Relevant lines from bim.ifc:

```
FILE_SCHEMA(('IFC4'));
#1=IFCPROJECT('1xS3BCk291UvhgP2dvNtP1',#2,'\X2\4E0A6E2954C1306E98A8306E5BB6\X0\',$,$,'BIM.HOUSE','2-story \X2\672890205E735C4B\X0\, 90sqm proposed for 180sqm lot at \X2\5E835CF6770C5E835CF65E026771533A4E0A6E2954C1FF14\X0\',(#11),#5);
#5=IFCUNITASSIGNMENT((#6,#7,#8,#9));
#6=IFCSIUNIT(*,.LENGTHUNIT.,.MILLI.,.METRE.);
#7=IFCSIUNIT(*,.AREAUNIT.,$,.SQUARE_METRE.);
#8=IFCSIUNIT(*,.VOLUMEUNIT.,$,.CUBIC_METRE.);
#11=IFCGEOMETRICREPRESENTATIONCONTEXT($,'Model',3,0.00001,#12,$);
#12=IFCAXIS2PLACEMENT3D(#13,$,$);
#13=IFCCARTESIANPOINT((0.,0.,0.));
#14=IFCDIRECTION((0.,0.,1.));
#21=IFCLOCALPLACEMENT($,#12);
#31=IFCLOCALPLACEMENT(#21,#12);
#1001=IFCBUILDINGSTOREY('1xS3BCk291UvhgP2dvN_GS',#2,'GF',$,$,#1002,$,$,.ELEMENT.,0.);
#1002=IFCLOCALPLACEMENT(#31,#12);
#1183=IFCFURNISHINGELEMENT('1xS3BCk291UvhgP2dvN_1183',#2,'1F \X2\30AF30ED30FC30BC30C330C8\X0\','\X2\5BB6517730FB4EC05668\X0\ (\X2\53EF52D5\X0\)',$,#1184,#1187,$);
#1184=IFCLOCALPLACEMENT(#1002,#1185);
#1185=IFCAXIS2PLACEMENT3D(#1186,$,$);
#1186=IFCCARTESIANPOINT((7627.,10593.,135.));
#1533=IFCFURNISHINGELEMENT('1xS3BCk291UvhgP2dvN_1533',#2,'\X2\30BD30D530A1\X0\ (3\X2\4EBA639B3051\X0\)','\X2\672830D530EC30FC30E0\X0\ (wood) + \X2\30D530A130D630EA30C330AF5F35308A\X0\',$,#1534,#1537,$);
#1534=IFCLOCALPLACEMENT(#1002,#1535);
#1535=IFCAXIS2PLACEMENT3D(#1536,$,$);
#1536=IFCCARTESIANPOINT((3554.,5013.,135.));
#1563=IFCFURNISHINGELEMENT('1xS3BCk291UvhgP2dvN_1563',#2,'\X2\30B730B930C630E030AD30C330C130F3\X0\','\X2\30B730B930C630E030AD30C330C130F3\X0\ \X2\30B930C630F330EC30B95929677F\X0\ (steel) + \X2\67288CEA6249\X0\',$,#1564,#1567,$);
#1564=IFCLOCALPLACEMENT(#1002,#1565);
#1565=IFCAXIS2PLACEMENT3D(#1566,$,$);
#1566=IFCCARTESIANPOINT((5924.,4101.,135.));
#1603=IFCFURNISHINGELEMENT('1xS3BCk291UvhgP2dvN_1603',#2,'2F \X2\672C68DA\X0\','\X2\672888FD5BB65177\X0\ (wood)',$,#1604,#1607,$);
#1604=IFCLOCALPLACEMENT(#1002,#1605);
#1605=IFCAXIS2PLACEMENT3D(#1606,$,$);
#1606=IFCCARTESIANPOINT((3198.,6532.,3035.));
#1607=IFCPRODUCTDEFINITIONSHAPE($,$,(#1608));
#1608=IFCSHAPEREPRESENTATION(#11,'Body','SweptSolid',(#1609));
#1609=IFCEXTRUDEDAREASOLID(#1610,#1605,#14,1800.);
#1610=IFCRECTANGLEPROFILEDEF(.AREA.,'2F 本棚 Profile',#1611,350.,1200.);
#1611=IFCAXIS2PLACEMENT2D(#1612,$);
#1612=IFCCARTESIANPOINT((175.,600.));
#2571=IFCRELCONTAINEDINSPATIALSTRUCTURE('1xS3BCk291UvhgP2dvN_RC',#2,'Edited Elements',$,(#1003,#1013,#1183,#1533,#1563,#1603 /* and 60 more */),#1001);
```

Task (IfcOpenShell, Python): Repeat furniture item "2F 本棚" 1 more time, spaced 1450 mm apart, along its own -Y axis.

```python
import ifcopenshell
import ifcopenshell.api.geometry
import ifcopenshell.api.root
import ifcopenshell.util.element
import ifcopenshell.util.placement
import ifcopenshell.util.unit

model = ifcopenshell.open("bim.ifc")
unit_scale = ifcopenshell.util.unit.calculate_unit_scale(model)


def reuse_history(source, copy):
    """copy_class also copies each property set's owner history, people and application; keep the originals."""
    for rel in copy.IsDefinedBy:
        if rel.is_a("IfcRelDefinesByProperties") and (history := rel.RelatingPropertyDefinition.OwnerHistory):
            rel.RelatingPropertyDefinition.OwnerHistory = source.OwnerHistory
            ifcopenshell.util.element.remove_deep2(model, history)


source = model.by_id(1603)
base = ifcopenshell.util.placement.get_local_placement(source.ObjectPlacement)
step = -base[:3, 1] * 1.45 / unit_scale

for i in range(1, 2):
    copy = ifcopenshell.api.root.copy_class(model, product=source)
    copy.Representation = ifcopenshell.util.element.copy_deep(
        model, source.Representation, exclude=["IfcGeometricRepresentationContext", "IfcRepresentationMap"]
    )
    reuse_history(source, copy)
    matrix = base.copy()
    matrix[:3, 3] += i * step
    print("added at", matrix[:3, 3].round(3) + 0.0)
    ifcopenshell.api.geometry.edit_object_placement(model, product=copy, matrix=matrix, is_si=False)

model.write("bim_v2.ifc")
```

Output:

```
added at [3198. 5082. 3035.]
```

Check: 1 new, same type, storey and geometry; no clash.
